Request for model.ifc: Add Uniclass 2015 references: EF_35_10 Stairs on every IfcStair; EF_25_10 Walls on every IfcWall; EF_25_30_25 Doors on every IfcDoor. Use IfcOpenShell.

First a look at what the model holds.

```python
import ifcopenshell

model = ifcopenshell.open("model.ifc")
print(model.schema)
print("classifications:", [c.Name for c in model.by_type("IfcClassification")])
for ifc_class in ("IfcDoor", "IfcRoof", "IfcStair", "IfcWall", "IfcWindow"):
    print(ifc_class, len(model.by_type(ifc_class)))
```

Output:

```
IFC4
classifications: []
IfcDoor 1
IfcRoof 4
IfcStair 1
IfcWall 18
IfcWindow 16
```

```python
import ifcopenshell
import ifcopenshell.api.classification

model = ifcopenshell.open("model.ifc")

system = ifcopenshell.api.classification.add_classification(model, classification="Uniclass 2015")

codes = {
    "IfcStair": ("EF_35_10", "Stairs"),
    "IfcWall": ("EF_25_10", "Walls"),
    "IfcDoor": ("EF_25_30_25", "Doors"),
}
for ifc_class, (code, name) in codes.items():
    products = model.by_type(ifc_class)
    ifcopenshell.api.classification.add_reference(
        model, products=products, classification=system, identification=code, name=name
    )
    print(code, len(products))

model.write("model_edited.ifc")
```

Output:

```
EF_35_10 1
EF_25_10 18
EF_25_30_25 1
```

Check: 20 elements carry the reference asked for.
